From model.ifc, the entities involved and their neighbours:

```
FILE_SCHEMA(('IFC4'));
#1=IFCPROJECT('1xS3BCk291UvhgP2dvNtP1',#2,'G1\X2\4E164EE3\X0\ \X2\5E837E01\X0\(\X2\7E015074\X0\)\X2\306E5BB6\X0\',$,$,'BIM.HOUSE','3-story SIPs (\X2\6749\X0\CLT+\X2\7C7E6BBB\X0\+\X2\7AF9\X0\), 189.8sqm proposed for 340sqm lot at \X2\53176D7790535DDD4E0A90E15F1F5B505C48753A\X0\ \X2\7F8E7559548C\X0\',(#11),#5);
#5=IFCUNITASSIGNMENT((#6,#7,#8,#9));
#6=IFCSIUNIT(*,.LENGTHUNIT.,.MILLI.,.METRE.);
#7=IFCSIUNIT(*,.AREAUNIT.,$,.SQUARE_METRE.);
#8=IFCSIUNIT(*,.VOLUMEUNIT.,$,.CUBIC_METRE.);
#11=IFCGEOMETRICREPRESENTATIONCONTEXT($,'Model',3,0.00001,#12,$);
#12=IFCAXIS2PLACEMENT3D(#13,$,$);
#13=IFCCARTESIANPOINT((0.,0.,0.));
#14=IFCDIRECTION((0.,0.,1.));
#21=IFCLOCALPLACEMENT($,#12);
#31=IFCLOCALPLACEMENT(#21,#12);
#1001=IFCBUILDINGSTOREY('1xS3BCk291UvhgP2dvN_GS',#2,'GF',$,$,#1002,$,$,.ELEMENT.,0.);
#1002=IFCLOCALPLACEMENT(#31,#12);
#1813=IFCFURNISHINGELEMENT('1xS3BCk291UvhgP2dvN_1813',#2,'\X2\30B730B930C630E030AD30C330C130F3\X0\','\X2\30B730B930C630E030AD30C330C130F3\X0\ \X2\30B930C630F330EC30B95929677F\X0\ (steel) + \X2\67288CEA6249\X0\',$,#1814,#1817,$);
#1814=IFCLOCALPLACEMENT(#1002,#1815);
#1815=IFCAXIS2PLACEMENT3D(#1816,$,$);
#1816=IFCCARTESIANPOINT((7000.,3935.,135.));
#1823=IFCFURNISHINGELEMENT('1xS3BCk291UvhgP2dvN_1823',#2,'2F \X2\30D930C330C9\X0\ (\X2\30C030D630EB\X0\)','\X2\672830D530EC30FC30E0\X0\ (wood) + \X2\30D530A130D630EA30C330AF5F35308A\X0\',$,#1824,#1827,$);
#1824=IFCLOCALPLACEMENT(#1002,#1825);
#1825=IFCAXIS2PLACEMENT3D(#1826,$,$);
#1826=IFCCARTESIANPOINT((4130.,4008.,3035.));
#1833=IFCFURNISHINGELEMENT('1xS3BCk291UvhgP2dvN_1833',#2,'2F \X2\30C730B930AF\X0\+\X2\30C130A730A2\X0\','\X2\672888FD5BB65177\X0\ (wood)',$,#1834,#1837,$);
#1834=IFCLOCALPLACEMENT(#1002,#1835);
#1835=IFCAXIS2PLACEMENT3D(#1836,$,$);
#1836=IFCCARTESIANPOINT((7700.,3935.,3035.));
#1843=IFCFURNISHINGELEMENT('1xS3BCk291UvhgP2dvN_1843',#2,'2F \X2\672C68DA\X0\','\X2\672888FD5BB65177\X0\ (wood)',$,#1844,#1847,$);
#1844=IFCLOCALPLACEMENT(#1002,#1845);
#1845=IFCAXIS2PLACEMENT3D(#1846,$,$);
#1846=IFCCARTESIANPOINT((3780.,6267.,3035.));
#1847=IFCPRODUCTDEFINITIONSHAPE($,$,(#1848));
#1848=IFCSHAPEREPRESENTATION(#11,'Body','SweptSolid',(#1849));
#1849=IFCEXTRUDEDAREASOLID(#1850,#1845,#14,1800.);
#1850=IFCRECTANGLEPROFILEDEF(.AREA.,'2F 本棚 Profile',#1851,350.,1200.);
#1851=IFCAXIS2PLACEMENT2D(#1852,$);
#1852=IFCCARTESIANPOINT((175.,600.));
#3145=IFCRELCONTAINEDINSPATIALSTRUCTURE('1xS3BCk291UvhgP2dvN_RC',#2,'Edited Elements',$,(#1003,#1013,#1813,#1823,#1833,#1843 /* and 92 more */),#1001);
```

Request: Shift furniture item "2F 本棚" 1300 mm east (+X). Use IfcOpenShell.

```python
import ifcopenshell
import ifcopenshell.api.geometry
import ifcopenshell.util.placement

model = ifcopenshell.open("model.ifc")

item = model.by_id(1843)
matrix = ifcopenshell.util.placement.get_local_placement(item.ObjectPlacement)
matrix[0, 3] += 1300.0
ifcopenshell.api.geometry.edit_object_placement(model, product=item, matrix=matrix, is_si=False)

print(ifcopenshell.util.placement.get_local_placement(item.ObjectPlacement).round(3) + 0.0)

model.write("model_rev.ifc")
```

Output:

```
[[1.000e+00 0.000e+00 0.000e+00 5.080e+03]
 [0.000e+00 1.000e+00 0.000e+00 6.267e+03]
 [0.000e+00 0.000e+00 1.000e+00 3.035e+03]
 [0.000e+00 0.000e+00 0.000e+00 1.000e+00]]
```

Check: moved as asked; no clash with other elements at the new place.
